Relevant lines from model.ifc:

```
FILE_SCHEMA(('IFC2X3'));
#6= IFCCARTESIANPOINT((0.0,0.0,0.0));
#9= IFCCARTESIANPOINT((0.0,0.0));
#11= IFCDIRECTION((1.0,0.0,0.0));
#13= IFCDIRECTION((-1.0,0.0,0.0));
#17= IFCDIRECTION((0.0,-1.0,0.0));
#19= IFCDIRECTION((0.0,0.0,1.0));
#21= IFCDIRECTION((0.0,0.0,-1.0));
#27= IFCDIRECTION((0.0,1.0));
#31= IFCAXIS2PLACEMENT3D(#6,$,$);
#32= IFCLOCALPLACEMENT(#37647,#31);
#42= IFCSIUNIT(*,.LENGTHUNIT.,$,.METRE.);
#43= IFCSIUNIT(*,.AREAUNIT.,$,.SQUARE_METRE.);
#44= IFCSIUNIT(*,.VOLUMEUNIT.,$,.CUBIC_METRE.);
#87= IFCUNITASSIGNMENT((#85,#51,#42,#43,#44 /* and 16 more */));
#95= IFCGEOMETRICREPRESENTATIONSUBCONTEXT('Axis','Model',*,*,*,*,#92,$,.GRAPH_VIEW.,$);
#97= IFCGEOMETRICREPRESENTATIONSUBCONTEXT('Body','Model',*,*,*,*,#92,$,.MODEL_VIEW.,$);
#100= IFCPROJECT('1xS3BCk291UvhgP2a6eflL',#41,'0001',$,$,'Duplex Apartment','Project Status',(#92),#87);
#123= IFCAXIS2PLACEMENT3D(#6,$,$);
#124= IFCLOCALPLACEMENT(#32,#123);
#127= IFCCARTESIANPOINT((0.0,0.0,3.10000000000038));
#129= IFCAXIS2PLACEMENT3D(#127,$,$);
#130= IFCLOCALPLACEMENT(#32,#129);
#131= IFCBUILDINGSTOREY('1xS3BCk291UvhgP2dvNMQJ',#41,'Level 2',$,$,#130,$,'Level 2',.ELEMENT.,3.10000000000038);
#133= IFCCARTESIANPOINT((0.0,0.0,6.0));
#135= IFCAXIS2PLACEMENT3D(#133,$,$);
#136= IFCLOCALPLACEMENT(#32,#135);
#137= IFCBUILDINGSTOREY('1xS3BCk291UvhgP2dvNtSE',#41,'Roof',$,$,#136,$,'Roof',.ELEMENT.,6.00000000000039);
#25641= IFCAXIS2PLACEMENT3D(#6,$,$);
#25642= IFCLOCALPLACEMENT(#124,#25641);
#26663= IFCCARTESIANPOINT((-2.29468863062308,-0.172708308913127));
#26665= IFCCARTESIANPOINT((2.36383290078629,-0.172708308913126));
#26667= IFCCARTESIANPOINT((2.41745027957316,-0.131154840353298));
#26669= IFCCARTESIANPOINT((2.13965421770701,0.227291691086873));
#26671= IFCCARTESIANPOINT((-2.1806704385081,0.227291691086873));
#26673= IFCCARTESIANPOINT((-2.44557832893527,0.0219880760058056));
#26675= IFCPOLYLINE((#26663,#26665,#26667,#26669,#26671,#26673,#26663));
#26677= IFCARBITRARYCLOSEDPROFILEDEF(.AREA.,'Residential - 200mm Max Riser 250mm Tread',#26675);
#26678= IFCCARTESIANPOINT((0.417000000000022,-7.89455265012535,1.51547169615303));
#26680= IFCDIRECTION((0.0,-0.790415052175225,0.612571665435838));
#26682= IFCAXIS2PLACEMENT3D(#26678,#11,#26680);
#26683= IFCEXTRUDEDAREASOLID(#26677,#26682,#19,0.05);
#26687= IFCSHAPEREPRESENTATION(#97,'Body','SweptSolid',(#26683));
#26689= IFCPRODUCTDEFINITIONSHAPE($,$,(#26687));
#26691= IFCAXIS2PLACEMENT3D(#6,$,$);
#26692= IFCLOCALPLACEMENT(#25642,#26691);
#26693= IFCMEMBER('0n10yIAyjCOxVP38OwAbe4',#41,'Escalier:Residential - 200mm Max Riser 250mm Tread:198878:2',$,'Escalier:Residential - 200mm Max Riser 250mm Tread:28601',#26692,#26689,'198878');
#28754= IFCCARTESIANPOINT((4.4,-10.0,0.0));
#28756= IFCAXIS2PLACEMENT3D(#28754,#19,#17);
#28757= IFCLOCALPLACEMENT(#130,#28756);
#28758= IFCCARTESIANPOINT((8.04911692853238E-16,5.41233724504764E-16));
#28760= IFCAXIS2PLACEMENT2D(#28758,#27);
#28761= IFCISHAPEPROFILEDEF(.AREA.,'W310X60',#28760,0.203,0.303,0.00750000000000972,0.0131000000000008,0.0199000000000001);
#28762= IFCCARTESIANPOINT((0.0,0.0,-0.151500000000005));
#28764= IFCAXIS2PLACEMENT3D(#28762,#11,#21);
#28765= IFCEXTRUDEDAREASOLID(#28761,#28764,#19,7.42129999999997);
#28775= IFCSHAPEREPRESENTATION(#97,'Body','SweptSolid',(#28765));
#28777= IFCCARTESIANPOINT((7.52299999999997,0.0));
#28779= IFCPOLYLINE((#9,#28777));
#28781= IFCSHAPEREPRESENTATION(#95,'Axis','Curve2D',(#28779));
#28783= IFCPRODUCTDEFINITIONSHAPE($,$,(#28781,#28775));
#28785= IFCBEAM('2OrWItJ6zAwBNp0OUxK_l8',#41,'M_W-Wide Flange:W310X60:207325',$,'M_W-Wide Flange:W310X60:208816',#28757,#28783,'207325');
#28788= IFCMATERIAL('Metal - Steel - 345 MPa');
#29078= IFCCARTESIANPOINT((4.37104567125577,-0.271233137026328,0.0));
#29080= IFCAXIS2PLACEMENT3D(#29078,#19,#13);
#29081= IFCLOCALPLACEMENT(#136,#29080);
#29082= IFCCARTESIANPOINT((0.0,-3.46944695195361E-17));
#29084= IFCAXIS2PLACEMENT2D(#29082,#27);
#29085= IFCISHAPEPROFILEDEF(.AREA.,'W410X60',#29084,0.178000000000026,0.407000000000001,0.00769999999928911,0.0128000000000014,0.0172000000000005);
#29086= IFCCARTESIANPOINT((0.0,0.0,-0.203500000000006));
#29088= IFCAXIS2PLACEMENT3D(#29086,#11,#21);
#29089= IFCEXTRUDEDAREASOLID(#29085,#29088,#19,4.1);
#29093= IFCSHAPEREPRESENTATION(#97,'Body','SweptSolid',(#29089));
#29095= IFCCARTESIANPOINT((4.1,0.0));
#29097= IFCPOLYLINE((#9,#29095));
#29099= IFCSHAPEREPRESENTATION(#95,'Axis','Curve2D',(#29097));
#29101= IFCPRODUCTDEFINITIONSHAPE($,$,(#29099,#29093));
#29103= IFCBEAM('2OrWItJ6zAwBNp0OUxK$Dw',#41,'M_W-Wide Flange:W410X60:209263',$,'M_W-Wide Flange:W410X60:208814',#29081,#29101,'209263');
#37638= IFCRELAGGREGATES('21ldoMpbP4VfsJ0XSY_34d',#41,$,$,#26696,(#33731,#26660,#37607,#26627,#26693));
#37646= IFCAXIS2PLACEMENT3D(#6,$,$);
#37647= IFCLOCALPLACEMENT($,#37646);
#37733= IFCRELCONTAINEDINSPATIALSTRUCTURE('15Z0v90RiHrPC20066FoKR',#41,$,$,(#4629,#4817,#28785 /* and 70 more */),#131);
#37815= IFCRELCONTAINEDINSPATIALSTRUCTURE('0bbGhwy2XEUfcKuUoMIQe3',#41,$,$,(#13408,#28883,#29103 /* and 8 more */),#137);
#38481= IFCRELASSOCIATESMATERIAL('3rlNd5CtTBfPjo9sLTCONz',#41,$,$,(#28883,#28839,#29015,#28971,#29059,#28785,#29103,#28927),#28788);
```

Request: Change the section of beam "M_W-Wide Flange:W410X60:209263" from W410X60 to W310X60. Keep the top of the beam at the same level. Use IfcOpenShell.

```python
import ifcopenshell
import ifcopenshell.util.element
import ifcopenshell.util.representation

model = ifcopenshell.open("model.ifc")

member = model.by_guid("2OrWItJ6zAwBNp0OUxK$Dw")
source = next(p for p in model.by_type("IfcIShapeProfileDef") if p.ProfileName == "W310X60")

body = ifcopenshell.util.representation.get_representation(member, "Model", "Body")
solid = body.Items[0]
old_profile = solid.SweptArea

# Copy the section's sizes but keep this member's own profile position.
profile = ifcopenshell.util.element.copy(model, source)
# Profiles are centred, so shift by half the change in depth to hold the top.
shift = (old_profile.OverallDepth - profile.OverallDepth) / 2
x, y = old_profile.Position.Location.Coordinates
up = (-1.0, 0.0)  # upwards, in the solid's own plane
location = model.createIfcCartesianPoint((x + up[0] * shift, y + up[1] * shift))
profile.Position = model.createIfcAxis2Placement2D(location, old_profile.Position.RefDirection)
solid.SweptArea = profile
if not model.get_total_inverses(old_profile):
    ifcopenshell.util.element.remove_deep2(model, old_profile)
member.Name = member.Name.replace("W410X60", "W310X60")
member.ObjectType = member.ObjectType.replace("W410X60", "W310X60")

print(solid.SweptArea)

model.write("model_edited.ifc")
```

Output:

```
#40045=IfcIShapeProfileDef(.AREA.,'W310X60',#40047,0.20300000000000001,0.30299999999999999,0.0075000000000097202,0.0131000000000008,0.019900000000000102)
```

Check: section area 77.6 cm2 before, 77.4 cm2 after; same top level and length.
